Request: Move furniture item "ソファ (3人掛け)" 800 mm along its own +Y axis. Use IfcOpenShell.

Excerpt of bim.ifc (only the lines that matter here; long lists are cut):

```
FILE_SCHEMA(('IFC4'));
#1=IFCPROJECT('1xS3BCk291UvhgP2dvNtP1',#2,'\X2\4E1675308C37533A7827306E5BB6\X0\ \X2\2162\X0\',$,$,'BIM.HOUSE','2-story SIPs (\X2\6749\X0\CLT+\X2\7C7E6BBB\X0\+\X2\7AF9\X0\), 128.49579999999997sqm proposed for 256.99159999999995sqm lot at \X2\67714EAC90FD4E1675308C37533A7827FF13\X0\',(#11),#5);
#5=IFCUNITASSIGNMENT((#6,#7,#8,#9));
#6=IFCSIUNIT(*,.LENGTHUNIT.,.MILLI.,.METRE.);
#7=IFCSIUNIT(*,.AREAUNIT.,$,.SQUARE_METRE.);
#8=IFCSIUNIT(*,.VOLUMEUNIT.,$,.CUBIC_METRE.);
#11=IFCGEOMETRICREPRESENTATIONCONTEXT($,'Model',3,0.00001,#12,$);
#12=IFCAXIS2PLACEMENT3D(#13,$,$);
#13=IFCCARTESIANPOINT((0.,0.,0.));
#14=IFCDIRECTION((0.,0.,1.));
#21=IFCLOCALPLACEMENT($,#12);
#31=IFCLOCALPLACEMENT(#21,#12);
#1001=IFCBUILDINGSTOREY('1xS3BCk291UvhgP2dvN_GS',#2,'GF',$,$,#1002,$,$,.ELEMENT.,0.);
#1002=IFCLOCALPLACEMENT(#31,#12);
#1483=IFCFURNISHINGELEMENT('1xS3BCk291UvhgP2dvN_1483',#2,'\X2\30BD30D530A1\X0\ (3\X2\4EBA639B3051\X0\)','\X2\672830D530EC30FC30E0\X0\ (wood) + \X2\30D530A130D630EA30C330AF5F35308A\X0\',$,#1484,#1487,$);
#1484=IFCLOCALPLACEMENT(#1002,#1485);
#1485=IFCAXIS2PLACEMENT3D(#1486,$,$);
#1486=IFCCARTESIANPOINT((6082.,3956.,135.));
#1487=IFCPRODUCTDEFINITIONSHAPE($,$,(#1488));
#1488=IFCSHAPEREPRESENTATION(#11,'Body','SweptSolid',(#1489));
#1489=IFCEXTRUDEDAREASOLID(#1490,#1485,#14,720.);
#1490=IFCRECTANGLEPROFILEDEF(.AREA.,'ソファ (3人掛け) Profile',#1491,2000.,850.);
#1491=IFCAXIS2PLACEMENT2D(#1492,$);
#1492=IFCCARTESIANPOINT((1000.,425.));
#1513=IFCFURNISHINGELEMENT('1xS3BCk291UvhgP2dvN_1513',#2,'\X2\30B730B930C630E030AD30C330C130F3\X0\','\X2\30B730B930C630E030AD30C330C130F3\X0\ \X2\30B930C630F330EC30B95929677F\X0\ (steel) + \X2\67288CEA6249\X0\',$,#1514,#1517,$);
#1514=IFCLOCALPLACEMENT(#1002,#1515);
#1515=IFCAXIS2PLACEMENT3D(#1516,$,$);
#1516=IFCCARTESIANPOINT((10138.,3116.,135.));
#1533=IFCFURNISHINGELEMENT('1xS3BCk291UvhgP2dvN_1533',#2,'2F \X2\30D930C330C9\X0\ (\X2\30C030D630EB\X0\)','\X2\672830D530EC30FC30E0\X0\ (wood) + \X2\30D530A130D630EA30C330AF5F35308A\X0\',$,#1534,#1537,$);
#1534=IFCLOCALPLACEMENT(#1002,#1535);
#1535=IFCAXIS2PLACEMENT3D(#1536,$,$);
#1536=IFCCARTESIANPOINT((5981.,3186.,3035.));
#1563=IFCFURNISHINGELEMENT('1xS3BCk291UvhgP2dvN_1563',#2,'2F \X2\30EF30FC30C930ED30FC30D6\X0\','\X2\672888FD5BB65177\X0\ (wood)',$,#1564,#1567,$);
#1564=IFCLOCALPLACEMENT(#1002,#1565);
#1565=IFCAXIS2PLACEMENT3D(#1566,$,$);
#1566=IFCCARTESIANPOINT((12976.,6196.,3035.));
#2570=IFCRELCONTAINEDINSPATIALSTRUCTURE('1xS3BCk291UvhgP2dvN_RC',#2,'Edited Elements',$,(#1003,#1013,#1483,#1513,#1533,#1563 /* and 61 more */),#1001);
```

```python
import ifcopenshell
import ifcopenshell.api.geometry
import ifcopenshell.util.placement
import ifcopenshell.util.unit

model = ifcopenshell.open("bim.ifc")
unit_scale = ifcopenshell.util.unit.calculate_unit_scale(model)

item = model.by_guid("1xS3BCk291UvhgP2dvN_1483")
matrix = ifcopenshell.util.placement.get_local_placement(item.ObjectPlacement)
matrix[:3, 3] += matrix[:3, 1] * 0.8 / unit_scale
ifcopenshell.api.geometry.edit_object_placement(model, product=item, matrix=matrix, is_si=False)

print(ifcopenshell.util.placement.get_local_placement(item.ObjectPlacement).round(3) + 0.0)

model.write("bim_edited.ifc")
```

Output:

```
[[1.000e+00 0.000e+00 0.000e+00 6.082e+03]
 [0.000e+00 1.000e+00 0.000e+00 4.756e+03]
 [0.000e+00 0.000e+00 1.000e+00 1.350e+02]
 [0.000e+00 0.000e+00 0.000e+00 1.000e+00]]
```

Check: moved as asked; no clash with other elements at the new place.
